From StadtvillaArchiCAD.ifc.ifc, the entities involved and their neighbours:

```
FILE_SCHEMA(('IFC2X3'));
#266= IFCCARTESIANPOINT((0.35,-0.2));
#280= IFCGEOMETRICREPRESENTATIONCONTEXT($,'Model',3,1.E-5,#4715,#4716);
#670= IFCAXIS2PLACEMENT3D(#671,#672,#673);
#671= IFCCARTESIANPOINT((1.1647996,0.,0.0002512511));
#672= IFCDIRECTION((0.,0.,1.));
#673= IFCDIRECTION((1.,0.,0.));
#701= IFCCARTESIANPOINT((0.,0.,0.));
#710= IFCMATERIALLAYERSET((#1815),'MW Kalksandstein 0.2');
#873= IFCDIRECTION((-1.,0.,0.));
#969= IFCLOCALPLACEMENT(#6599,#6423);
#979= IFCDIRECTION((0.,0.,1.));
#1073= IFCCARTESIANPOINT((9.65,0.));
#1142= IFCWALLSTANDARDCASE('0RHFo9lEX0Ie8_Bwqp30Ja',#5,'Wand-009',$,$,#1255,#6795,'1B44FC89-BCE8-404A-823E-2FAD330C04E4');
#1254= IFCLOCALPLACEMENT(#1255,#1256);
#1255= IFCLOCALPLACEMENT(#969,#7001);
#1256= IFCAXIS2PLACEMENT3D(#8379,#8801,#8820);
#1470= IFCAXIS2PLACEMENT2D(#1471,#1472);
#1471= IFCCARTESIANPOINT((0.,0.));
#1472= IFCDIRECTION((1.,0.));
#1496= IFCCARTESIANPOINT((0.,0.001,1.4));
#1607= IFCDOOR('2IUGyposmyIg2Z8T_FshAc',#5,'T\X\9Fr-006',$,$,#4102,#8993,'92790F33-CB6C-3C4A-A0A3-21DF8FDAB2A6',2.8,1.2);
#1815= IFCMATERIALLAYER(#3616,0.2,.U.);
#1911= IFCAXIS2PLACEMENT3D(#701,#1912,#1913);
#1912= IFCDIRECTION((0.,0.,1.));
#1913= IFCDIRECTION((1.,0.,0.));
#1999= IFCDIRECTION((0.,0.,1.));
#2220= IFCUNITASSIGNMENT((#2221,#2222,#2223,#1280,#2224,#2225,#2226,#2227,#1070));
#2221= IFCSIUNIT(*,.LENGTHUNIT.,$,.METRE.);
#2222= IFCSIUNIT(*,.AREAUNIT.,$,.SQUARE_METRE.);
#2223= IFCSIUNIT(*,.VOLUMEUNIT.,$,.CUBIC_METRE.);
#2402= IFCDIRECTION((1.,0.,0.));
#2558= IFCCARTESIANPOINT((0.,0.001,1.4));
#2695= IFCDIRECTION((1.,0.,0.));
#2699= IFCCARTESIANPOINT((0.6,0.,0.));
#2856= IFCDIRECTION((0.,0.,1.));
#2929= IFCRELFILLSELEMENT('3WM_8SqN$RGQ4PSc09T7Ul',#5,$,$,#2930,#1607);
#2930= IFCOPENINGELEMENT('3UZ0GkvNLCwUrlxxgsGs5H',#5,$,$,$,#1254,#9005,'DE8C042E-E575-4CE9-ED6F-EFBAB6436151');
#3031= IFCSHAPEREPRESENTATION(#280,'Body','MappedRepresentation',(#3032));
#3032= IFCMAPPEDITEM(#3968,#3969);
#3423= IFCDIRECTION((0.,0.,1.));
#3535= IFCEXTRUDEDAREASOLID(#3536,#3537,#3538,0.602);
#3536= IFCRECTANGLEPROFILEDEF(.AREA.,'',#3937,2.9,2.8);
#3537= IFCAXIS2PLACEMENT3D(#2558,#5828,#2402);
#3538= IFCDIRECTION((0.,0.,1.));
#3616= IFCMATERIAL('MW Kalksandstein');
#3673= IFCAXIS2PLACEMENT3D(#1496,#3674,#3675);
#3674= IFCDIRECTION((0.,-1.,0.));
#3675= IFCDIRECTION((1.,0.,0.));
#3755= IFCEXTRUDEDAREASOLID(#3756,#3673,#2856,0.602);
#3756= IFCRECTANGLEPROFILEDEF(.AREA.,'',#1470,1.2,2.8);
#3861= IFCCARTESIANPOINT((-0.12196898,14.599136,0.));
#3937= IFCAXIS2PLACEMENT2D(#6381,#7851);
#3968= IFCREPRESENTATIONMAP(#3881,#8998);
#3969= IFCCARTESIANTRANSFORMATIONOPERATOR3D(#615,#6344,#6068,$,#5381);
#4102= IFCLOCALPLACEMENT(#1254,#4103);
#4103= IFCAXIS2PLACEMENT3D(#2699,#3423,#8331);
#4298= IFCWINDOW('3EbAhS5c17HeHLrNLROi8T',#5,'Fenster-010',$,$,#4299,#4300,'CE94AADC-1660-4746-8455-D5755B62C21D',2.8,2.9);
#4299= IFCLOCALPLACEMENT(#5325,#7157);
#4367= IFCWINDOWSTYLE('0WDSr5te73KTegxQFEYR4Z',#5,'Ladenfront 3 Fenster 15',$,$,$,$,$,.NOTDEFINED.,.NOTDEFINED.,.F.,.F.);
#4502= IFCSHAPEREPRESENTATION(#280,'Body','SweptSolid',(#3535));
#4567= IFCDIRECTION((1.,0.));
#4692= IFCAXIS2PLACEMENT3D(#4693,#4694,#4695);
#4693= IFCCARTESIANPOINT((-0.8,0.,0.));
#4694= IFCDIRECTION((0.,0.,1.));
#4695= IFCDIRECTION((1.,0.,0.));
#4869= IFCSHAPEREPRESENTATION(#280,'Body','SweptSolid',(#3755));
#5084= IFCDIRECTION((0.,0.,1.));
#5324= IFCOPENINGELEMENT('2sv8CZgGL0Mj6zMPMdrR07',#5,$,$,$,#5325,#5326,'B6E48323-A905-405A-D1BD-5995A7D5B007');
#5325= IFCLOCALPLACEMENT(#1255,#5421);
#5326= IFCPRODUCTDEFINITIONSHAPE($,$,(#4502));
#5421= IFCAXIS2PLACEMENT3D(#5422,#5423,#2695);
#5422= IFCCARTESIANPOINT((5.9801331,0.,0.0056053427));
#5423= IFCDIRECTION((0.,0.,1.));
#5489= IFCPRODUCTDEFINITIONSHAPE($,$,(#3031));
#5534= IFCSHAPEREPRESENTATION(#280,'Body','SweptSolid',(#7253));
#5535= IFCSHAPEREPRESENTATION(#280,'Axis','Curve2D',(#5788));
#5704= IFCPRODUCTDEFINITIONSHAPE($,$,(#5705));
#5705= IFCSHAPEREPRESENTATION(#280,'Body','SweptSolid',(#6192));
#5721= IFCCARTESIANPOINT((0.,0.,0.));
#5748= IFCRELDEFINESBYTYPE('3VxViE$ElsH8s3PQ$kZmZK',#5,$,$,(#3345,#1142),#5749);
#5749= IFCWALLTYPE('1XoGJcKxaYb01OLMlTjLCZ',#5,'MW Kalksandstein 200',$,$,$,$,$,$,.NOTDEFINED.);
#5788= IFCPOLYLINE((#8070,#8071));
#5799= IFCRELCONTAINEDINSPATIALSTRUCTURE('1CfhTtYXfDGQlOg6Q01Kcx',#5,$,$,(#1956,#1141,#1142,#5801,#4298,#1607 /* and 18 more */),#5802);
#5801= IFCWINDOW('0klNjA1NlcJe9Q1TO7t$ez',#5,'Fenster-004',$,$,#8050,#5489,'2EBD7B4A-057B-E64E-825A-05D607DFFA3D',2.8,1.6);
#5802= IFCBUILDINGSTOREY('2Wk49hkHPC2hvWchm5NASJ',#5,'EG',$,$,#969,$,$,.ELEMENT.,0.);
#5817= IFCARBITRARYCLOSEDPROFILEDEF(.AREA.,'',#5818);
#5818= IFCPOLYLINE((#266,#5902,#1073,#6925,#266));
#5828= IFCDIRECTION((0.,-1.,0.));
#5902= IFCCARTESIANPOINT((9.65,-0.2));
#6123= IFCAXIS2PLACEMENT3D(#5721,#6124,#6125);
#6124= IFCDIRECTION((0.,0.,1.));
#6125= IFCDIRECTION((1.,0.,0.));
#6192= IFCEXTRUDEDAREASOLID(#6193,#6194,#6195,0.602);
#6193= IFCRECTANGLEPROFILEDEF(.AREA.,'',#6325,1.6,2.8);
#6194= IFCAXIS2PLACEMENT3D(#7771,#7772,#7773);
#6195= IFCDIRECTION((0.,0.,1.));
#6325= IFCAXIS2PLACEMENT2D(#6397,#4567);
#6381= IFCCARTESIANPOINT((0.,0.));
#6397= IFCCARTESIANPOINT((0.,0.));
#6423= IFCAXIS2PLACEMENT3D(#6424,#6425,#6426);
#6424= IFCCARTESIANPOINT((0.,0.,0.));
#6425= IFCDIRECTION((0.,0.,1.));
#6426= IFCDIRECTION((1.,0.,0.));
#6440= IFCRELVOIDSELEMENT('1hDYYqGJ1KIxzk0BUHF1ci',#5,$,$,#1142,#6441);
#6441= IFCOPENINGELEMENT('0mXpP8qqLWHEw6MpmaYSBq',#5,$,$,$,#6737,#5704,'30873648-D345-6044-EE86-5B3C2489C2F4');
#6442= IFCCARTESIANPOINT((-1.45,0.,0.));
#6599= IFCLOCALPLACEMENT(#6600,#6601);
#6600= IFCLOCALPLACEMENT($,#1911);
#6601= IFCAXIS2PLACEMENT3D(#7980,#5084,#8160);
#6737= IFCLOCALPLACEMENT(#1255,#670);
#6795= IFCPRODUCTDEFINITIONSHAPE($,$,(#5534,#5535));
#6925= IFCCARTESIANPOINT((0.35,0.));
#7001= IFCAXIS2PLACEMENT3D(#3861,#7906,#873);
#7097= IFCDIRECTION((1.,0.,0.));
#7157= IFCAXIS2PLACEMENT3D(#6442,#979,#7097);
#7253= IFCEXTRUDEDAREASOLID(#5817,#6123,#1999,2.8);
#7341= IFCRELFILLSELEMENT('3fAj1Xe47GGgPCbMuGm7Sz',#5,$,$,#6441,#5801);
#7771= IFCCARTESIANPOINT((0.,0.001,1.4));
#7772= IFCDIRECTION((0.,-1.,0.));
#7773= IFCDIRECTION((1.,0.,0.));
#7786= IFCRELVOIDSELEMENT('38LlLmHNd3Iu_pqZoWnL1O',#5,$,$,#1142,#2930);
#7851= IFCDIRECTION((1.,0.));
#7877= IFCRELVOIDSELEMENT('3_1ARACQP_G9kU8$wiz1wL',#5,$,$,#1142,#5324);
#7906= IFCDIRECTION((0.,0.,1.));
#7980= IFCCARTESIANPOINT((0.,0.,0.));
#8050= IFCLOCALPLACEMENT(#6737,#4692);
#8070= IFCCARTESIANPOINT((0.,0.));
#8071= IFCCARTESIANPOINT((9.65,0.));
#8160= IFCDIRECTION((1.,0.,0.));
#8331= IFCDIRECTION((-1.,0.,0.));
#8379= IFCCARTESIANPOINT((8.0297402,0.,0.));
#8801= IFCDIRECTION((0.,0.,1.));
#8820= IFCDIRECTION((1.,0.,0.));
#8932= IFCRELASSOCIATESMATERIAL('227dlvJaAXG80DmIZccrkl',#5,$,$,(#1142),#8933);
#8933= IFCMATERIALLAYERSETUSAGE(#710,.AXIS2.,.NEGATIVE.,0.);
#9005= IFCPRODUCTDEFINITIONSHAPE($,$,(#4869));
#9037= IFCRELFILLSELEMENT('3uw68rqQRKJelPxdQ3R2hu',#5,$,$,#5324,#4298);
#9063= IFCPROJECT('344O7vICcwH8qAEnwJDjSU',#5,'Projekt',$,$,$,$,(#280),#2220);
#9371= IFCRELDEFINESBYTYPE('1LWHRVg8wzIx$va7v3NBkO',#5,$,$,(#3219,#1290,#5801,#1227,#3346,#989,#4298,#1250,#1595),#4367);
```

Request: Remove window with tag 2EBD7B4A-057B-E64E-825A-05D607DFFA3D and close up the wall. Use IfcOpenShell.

```python
import ifcopenshell
import ifcopenshell.api.feature
import ifcopenshell.api.root
import ifcopenshell.geom
import ifcopenshell.util.shape

model = ifcopenshell.open("StadtvillaArchiCAD.ifc.ifc")
settings = ifcopenshell.geom.settings()


def volume(element):
    """Net volume in cubic metres, openings subtracted."""
    shape = ifcopenshell.geom.create_shape(settings, element)
    return ifcopenshell.util.shape.get_volume(shape.geometry)


window = model.by_guid("0klNjA1NlcJe9Q1TO7t$ez")
opening = window.FillsVoids[0].RelatingOpeningElement
wall = opening.VoidsElements[0].RelatingBuildingElement
before = volume(wall)

ifcopenshell.api.root.remove_product(model, product=window)
ifcopenshell.api.feature.remove_feature(model, feature=opening)

after = volume(wall)

print(f"wall volume {before:.3f} -> {after:.3f} m3")

model.write("StadtvillaArchiCAD.ifc_updated.ifc")
```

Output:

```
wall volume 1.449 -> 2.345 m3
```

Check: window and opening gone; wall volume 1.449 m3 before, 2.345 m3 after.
